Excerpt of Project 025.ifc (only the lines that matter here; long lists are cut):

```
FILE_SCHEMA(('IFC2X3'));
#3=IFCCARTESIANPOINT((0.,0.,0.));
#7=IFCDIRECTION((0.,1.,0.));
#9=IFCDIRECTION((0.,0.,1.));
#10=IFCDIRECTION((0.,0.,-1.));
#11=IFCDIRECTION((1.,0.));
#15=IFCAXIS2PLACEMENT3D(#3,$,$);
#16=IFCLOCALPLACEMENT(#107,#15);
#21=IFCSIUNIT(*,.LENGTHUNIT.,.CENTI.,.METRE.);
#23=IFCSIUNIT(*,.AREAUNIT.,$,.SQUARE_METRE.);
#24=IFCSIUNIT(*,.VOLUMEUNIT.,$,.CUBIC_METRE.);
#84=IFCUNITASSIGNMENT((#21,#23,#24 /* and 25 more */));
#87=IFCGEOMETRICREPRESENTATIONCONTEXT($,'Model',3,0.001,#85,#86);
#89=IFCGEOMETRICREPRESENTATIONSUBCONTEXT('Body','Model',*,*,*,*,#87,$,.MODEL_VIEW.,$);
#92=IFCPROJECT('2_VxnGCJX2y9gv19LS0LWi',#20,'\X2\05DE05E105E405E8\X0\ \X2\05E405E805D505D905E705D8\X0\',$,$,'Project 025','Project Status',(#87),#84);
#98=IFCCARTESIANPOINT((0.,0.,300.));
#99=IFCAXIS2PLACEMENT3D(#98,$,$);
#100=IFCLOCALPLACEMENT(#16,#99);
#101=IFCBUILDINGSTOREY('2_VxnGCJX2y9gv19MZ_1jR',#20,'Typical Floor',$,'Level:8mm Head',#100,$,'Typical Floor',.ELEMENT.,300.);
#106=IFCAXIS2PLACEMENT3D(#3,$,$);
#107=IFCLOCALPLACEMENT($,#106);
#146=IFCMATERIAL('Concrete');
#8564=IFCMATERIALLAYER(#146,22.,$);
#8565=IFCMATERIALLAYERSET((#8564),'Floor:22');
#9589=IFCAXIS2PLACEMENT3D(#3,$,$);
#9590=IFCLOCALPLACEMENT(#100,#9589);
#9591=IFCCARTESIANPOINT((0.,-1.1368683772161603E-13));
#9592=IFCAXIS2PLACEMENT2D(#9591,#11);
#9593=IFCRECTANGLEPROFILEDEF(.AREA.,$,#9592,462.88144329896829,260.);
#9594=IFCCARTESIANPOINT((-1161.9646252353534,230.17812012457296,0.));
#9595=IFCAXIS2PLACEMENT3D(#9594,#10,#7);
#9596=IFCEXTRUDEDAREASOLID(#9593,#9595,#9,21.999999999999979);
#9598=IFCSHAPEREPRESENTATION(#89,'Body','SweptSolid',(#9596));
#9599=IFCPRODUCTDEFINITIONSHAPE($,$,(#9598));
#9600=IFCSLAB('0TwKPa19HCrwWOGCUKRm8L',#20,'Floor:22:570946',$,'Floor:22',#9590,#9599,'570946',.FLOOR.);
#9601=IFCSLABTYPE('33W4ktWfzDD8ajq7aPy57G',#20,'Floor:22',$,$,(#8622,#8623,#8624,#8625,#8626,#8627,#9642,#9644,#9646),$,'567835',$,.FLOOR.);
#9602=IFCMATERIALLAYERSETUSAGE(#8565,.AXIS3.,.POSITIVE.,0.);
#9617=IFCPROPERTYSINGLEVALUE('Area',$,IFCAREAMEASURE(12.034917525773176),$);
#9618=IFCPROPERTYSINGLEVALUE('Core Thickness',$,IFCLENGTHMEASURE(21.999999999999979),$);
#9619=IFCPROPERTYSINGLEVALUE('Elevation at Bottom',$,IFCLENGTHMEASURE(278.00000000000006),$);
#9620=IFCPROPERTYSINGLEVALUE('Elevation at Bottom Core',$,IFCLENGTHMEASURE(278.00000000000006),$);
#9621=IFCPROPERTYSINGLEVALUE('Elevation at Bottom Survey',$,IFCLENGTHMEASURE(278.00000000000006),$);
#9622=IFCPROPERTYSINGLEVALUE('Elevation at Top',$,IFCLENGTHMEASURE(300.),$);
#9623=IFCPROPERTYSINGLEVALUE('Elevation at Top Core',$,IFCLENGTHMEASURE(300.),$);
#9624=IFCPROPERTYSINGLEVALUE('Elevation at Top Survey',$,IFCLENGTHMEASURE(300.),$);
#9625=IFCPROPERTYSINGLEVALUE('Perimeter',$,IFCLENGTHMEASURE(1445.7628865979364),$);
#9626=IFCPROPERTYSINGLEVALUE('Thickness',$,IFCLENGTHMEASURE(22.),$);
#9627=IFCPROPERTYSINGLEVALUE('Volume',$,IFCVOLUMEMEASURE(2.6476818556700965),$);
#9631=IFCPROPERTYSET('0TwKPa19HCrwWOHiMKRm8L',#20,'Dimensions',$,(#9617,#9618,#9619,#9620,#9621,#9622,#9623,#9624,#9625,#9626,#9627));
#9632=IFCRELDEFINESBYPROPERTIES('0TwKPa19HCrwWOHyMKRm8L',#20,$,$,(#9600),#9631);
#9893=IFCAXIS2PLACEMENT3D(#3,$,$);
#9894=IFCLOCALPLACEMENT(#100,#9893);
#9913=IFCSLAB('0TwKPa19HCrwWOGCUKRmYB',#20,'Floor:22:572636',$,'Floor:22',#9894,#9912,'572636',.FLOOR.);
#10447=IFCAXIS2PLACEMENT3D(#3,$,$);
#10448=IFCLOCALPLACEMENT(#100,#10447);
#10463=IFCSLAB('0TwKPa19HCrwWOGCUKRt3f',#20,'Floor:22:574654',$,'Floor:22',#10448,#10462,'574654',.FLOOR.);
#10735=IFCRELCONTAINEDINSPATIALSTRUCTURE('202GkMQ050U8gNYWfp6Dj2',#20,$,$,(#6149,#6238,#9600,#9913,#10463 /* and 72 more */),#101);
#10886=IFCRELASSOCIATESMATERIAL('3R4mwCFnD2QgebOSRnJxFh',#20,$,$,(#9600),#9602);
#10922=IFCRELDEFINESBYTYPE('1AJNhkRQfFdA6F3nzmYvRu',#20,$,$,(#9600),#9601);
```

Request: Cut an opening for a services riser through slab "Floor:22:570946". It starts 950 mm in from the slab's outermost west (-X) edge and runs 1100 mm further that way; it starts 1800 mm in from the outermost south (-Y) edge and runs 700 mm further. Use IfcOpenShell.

```python
import numpy as np
import ifcopenshell
import ifcopenshell.api.feature
import ifcopenshell.api.geometry
import ifcopenshell.api.pset
import ifcopenshell.api.root
import ifcopenshell.geom
import ifcopenshell.util.element
import ifcopenshell.util.placement
import ifcopenshell.util.representation
import ifcopenshell.util.shape
import ifcopenshell.util.unit

model = ifcopenshell.open("Project 025.ifc")
unit_scale = ifcopenshell.util.unit.calculate_unit_scale(model)
area_scale = ifcopenshell.util.unit.calculate_unit_scale(model, "AREAUNIT")
volume_scale = ifcopenshell.util.unit.calculate_unit_scale(model, "VOLUMEUNIT")
settings = ifcopenshell.geom.settings()


def volume(element):
    """Net volume in cubic metres, openings subtracted."""
    shape = ifcopenshell.geom.create_shape(settings, element)
    return ifcopenshell.util.shape.get_volume(shape.geometry)


slab = model.by_guid("0TwKPa19HCrwWOGCUKRm8L")
before = volume(slab)

# Extent in the slab's own axes, in metres. The edges named are its -X and -Y sides.
slab_shape = ifcopenshell.geom.create_shape(settings, slab)
vertices = ifcopenshell.util.shape.get_vertices(slab_shape.geometry)
x_min, y_min, bottom = vertices.min(axis=0)
top = vertices[:, 2].max()

opening = ifcopenshell.api.root.create_entity(model, ifc_class="IfcOpeningElement", name="Services riser opening")
context = ifcopenshell.util.representation.get_context(model, "Model", "Body", "MODEL_VIEW")
width, depth = 1.1, 0.7
outline = [(0.0, 0.0), (width, 0.0), (width, depth), (0.0, depth), (0.0, 0.0)]
# Overshoot both faces by 50 mm so the cut is clean.
shape = ifcopenshell.api.geometry.add_slab_representation(
    model, context=context, depth=top - bottom + 0.1, polyline=outline
)
ifcopenshell.api.geometry.assign_representation(model, product=opening, representation=shape)

matrix = ifcopenshell.util.placement.get_local_placement(slab.ObjectPlacement)
matrix[:, 3] = matrix @ np.append(np.array([x_min + 0.95, y_min + 1.8, bottom - 0.05]) / unit_scale, 1.0)
ifcopenshell.api.geometry.edit_object_placement(model, product=opening, matrix=matrix, is_si=False)
ifcopenshell.api.feature.add_feature(model, feature=opening, element=slab)

after = volume(slab)

# Update the slab's stored quantities.
pset = model.by_id(ifcopenshell.util.element.get_pset(slab, "Dimensions", should_inherit=False)["id"])
ifcopenshell.api.pset.edit_pset(model, pset=pset, properties={
    "Area": model.create_entity("IfcAreaMeasure", after / (top - bottom) / area_scale),
    "Volume": model.create_entity("IfcVolumeMeasure", after / volume_scale),
})

print(f"slab volume {before:.3f} -> {after:.3f} m3")

model.write("Project 025_updated.ifc")
```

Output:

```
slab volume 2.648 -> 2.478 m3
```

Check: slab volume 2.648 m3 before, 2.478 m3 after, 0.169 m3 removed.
